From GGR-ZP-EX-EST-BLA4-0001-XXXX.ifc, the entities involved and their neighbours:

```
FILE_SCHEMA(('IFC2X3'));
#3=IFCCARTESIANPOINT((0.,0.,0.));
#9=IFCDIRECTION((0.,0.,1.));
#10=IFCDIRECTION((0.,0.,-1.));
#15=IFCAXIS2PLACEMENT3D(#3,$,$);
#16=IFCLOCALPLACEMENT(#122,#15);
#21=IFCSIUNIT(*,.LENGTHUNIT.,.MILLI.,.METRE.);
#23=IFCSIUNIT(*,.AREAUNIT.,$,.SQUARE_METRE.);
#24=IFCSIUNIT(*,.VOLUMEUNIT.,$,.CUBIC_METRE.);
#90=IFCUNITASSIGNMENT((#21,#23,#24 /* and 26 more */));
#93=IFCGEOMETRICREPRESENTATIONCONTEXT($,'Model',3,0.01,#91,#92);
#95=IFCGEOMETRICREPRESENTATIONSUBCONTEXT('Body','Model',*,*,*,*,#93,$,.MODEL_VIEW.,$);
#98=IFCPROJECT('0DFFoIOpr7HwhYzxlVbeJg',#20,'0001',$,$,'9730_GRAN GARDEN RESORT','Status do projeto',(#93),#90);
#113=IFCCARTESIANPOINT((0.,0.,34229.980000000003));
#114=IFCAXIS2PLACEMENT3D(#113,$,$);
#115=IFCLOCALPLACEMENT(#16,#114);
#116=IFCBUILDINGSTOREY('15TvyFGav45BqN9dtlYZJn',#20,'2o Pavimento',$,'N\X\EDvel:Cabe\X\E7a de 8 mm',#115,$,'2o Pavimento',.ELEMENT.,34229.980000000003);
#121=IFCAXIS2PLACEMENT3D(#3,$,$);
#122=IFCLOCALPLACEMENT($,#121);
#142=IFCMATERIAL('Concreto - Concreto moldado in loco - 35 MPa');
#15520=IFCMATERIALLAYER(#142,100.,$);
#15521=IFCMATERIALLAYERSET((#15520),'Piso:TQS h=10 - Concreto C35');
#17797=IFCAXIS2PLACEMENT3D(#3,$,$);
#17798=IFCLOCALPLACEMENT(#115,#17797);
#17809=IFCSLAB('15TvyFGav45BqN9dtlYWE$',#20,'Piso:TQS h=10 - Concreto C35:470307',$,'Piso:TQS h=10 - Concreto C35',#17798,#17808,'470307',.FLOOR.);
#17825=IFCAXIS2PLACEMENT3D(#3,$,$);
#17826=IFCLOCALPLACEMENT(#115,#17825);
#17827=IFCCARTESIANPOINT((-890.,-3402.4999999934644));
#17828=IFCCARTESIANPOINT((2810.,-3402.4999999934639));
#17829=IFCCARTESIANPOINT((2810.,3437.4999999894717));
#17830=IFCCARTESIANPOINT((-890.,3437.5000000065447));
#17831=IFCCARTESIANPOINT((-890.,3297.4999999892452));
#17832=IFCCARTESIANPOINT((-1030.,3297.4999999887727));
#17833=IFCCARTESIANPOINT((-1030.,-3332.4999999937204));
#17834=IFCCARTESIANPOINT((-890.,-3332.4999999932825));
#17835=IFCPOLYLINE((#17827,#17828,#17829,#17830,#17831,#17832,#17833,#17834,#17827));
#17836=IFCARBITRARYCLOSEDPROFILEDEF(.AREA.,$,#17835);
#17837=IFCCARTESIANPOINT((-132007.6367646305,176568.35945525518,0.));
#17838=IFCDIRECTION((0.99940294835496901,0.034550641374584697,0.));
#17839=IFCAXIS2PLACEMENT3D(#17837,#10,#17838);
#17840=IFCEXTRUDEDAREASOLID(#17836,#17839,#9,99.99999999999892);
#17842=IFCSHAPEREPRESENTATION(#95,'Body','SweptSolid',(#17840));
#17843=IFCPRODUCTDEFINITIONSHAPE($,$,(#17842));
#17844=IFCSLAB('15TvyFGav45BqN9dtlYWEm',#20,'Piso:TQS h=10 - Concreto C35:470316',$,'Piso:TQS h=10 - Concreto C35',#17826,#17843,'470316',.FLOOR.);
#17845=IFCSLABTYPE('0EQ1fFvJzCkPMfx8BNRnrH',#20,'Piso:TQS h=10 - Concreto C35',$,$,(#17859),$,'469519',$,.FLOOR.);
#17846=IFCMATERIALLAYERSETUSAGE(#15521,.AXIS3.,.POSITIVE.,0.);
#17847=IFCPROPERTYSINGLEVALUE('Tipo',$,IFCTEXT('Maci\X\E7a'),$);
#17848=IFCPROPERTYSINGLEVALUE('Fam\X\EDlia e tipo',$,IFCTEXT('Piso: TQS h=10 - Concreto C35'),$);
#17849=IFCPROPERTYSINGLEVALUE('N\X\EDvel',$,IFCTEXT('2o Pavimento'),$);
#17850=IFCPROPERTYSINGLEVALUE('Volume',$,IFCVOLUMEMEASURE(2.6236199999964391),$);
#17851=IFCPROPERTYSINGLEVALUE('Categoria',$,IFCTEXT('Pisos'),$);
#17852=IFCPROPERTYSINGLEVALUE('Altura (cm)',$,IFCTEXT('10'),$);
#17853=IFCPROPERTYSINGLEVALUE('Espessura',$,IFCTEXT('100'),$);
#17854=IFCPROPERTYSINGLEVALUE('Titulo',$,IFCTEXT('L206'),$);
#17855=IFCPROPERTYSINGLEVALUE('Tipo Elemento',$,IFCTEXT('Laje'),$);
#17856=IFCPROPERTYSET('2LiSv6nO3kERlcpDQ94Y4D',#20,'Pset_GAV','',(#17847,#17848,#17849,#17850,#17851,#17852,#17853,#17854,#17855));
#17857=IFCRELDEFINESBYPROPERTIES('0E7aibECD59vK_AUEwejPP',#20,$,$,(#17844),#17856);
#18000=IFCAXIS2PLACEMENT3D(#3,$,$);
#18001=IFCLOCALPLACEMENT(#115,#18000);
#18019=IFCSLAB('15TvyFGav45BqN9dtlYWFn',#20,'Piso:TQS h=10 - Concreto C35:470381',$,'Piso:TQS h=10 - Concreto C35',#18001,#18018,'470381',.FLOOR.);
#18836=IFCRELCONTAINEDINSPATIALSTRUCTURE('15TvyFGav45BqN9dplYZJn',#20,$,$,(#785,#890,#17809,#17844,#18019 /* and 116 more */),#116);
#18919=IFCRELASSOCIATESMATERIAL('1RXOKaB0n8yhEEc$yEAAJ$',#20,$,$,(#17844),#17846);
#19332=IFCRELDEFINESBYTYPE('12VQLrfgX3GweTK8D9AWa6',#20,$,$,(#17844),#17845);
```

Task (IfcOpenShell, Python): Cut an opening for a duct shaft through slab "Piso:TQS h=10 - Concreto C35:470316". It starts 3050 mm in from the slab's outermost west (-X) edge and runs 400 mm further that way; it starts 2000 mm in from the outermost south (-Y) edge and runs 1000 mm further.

```python
import numpy as np
import ifcopenshell
import ifcopenshell.api.feature
import ifcopenshell.api.geometry
import ifcopenshell.api.pset
import ifcopenshell.api.root
import ifcopenshell.geom
import ifcopenshell.util.element
import ifcopenshell.util.placement
import ifcopenshell.util.representation
import ifcopenshell.util.shape
import ifcopenshell.util.unit

model = ifcopenshell.open("GGR-ZP-EX-EST-BLA4-0001-XXXX.ifc")
unit_scale = ifcopenshell.util.unit.calculate_unit_scale(model)
volume_scale = ifcopenshell.util.unit.calculate_unit_scale(model, "VOLUMEUNIT")
settings = ifcopenshell.geom.settings()


def volume(element):
    """Net volume in cubic metres, openings subtracted."""
    shape = ifcopenshell.geom.create_shape(settings, element)
    return ifcopenshell.util.shape.get_volume(shape.geometry)


slab = model.by_guid("15TvyFGav45BqN9dtlYWEm")
before = volume(slab)

# Extent in the slab's own axes, in metres. The edges named are its -X and -Y sides.
slab_shape = ifcopenshell.geom.create_shape(settings, slab)
vertices = ifcopenshell.util.shape.get_vertices(slab_shape.geometry)
x_min, y_min, bottom = vertices.min(axis=0)
top = vertices[:, 2].max()

opening = ifcopenshell.api.root.create_entity(model, ifc_class="IfcOpeningElement", name="Duct shaft opening")
context = ifcopenshell.util.representation.get_context(model, "Model", "Body", "MODEL_VIEW")
width, depth = 0.4, 1
outline = [(0.0, 0.0), (width, 0.0), (width, depth), (0.0, depth), (0.0, 0.0)]
# Overshoot both faces by 50 mm so the cut is clean.
shape = ifcopenshell.api.geometry.add_slab_representation(
    model, context=context, depth=top - bottom + 0.1, polyline=outline
)
ifcopenshell.api.geometry.assign_representation(model, product=opening, representation=shape)

matrix = ifcopenshell.util.placement.get_local_placement(slab.ObjectPlacement)
matrix[:, 3] = matrix @ np.append(np.array([x_min + 3.05, y_min + 2, bottom - 0.05]) / unit_scale, 1.0)
ifcopenshell.api.geometry.edit_object_placement(model, product=opening, matrix=matrix, is_si=False)
ifcopenshell.api.feature.add_feature(model, feature=opening, element=slab)

after = volume(slab)

# Update the slab's stored quantities.
pset = model.by_id(ifcopenshell.util.element.get_pset(slab, "Pset_GAV", should_inherit=False)["id"])
ifcopenshell.api.pset.edit_pset(model, pset=pset, properties={
    "Volume": model.create_entity("IfcVolumeMeasure", after / volume_scale),
})

print(f"slab volume {before:.3f} -> {after:.3f} m3")

model.write("GGR-ZP-EX-EST-BLA4-0001-XXXX_edited.ifc")
```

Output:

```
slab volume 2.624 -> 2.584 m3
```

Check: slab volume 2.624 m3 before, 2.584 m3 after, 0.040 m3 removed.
